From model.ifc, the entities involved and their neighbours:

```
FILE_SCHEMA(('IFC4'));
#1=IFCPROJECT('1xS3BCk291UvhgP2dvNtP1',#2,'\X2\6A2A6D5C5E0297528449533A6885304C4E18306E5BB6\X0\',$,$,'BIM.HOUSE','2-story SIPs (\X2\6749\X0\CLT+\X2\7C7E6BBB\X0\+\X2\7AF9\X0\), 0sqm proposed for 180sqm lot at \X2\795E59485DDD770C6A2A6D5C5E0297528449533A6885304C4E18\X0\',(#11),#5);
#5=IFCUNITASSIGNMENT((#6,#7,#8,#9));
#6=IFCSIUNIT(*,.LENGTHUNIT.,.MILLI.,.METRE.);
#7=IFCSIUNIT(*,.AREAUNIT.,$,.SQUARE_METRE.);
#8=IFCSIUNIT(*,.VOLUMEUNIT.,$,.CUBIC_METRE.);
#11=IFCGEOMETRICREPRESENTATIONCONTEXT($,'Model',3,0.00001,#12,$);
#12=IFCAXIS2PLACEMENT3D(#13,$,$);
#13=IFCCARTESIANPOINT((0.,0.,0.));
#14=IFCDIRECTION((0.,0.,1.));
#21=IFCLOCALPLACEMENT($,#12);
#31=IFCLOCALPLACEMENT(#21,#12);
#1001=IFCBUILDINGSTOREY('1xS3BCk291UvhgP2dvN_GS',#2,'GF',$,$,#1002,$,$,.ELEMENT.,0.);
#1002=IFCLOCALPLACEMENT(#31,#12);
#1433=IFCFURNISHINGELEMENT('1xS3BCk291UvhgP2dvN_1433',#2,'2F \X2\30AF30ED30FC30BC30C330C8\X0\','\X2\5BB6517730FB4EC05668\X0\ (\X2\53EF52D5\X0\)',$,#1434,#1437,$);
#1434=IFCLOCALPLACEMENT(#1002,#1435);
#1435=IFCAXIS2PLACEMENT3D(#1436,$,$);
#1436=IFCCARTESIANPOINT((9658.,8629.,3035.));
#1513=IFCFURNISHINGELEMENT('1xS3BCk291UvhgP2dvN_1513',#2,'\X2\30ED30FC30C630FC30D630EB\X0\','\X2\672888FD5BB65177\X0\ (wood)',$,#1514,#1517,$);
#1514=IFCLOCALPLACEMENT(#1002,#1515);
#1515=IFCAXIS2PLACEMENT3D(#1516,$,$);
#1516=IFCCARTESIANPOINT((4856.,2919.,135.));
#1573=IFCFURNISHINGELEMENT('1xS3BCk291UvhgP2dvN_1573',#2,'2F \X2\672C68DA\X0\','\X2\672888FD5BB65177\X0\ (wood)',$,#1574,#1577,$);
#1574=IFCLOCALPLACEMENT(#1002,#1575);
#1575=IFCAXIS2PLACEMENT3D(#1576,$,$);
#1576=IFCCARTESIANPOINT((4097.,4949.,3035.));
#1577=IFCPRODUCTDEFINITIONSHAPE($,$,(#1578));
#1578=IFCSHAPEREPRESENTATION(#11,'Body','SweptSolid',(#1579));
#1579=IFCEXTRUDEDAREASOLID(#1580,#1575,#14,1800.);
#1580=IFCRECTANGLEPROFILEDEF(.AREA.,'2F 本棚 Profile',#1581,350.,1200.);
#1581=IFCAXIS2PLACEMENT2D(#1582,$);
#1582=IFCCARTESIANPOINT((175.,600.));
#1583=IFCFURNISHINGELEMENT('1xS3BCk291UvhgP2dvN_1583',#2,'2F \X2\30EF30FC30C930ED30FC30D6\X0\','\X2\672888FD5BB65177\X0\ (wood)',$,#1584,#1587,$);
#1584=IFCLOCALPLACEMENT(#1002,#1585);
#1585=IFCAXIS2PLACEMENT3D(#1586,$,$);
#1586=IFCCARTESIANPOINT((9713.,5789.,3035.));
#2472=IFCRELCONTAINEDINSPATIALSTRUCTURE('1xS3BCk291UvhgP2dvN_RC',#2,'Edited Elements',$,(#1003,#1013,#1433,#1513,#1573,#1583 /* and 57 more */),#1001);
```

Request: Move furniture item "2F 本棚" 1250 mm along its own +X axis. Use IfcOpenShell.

```python
import ifcopenshell
import ifcopenshell.api.geometry
import ifcopenshell.util.placement

model = ifcopenshell.open("model.ifc")

item = model.by_guid("1xS3BCk291UvhgP2dvN_1573")
matrix = ifcopenshell.util.placement.get_local_placement(item.ObjectPlacement)
matrix[:3, 3] += matrix[:3, 0] * 1250.0
ifcopenshell.api.geometry.edit_object_placement(model, product=item, matrix=matrix, is_si=False)

print(ifcopenshell.util.placement.get_local_placement(item.ObjectPlacement).round(3) + 0.0)

model.write("model_v2.ifc")
```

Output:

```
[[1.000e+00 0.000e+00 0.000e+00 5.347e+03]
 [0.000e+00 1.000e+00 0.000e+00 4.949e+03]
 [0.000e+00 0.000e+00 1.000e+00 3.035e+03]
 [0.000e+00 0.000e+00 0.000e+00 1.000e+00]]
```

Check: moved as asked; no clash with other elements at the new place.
